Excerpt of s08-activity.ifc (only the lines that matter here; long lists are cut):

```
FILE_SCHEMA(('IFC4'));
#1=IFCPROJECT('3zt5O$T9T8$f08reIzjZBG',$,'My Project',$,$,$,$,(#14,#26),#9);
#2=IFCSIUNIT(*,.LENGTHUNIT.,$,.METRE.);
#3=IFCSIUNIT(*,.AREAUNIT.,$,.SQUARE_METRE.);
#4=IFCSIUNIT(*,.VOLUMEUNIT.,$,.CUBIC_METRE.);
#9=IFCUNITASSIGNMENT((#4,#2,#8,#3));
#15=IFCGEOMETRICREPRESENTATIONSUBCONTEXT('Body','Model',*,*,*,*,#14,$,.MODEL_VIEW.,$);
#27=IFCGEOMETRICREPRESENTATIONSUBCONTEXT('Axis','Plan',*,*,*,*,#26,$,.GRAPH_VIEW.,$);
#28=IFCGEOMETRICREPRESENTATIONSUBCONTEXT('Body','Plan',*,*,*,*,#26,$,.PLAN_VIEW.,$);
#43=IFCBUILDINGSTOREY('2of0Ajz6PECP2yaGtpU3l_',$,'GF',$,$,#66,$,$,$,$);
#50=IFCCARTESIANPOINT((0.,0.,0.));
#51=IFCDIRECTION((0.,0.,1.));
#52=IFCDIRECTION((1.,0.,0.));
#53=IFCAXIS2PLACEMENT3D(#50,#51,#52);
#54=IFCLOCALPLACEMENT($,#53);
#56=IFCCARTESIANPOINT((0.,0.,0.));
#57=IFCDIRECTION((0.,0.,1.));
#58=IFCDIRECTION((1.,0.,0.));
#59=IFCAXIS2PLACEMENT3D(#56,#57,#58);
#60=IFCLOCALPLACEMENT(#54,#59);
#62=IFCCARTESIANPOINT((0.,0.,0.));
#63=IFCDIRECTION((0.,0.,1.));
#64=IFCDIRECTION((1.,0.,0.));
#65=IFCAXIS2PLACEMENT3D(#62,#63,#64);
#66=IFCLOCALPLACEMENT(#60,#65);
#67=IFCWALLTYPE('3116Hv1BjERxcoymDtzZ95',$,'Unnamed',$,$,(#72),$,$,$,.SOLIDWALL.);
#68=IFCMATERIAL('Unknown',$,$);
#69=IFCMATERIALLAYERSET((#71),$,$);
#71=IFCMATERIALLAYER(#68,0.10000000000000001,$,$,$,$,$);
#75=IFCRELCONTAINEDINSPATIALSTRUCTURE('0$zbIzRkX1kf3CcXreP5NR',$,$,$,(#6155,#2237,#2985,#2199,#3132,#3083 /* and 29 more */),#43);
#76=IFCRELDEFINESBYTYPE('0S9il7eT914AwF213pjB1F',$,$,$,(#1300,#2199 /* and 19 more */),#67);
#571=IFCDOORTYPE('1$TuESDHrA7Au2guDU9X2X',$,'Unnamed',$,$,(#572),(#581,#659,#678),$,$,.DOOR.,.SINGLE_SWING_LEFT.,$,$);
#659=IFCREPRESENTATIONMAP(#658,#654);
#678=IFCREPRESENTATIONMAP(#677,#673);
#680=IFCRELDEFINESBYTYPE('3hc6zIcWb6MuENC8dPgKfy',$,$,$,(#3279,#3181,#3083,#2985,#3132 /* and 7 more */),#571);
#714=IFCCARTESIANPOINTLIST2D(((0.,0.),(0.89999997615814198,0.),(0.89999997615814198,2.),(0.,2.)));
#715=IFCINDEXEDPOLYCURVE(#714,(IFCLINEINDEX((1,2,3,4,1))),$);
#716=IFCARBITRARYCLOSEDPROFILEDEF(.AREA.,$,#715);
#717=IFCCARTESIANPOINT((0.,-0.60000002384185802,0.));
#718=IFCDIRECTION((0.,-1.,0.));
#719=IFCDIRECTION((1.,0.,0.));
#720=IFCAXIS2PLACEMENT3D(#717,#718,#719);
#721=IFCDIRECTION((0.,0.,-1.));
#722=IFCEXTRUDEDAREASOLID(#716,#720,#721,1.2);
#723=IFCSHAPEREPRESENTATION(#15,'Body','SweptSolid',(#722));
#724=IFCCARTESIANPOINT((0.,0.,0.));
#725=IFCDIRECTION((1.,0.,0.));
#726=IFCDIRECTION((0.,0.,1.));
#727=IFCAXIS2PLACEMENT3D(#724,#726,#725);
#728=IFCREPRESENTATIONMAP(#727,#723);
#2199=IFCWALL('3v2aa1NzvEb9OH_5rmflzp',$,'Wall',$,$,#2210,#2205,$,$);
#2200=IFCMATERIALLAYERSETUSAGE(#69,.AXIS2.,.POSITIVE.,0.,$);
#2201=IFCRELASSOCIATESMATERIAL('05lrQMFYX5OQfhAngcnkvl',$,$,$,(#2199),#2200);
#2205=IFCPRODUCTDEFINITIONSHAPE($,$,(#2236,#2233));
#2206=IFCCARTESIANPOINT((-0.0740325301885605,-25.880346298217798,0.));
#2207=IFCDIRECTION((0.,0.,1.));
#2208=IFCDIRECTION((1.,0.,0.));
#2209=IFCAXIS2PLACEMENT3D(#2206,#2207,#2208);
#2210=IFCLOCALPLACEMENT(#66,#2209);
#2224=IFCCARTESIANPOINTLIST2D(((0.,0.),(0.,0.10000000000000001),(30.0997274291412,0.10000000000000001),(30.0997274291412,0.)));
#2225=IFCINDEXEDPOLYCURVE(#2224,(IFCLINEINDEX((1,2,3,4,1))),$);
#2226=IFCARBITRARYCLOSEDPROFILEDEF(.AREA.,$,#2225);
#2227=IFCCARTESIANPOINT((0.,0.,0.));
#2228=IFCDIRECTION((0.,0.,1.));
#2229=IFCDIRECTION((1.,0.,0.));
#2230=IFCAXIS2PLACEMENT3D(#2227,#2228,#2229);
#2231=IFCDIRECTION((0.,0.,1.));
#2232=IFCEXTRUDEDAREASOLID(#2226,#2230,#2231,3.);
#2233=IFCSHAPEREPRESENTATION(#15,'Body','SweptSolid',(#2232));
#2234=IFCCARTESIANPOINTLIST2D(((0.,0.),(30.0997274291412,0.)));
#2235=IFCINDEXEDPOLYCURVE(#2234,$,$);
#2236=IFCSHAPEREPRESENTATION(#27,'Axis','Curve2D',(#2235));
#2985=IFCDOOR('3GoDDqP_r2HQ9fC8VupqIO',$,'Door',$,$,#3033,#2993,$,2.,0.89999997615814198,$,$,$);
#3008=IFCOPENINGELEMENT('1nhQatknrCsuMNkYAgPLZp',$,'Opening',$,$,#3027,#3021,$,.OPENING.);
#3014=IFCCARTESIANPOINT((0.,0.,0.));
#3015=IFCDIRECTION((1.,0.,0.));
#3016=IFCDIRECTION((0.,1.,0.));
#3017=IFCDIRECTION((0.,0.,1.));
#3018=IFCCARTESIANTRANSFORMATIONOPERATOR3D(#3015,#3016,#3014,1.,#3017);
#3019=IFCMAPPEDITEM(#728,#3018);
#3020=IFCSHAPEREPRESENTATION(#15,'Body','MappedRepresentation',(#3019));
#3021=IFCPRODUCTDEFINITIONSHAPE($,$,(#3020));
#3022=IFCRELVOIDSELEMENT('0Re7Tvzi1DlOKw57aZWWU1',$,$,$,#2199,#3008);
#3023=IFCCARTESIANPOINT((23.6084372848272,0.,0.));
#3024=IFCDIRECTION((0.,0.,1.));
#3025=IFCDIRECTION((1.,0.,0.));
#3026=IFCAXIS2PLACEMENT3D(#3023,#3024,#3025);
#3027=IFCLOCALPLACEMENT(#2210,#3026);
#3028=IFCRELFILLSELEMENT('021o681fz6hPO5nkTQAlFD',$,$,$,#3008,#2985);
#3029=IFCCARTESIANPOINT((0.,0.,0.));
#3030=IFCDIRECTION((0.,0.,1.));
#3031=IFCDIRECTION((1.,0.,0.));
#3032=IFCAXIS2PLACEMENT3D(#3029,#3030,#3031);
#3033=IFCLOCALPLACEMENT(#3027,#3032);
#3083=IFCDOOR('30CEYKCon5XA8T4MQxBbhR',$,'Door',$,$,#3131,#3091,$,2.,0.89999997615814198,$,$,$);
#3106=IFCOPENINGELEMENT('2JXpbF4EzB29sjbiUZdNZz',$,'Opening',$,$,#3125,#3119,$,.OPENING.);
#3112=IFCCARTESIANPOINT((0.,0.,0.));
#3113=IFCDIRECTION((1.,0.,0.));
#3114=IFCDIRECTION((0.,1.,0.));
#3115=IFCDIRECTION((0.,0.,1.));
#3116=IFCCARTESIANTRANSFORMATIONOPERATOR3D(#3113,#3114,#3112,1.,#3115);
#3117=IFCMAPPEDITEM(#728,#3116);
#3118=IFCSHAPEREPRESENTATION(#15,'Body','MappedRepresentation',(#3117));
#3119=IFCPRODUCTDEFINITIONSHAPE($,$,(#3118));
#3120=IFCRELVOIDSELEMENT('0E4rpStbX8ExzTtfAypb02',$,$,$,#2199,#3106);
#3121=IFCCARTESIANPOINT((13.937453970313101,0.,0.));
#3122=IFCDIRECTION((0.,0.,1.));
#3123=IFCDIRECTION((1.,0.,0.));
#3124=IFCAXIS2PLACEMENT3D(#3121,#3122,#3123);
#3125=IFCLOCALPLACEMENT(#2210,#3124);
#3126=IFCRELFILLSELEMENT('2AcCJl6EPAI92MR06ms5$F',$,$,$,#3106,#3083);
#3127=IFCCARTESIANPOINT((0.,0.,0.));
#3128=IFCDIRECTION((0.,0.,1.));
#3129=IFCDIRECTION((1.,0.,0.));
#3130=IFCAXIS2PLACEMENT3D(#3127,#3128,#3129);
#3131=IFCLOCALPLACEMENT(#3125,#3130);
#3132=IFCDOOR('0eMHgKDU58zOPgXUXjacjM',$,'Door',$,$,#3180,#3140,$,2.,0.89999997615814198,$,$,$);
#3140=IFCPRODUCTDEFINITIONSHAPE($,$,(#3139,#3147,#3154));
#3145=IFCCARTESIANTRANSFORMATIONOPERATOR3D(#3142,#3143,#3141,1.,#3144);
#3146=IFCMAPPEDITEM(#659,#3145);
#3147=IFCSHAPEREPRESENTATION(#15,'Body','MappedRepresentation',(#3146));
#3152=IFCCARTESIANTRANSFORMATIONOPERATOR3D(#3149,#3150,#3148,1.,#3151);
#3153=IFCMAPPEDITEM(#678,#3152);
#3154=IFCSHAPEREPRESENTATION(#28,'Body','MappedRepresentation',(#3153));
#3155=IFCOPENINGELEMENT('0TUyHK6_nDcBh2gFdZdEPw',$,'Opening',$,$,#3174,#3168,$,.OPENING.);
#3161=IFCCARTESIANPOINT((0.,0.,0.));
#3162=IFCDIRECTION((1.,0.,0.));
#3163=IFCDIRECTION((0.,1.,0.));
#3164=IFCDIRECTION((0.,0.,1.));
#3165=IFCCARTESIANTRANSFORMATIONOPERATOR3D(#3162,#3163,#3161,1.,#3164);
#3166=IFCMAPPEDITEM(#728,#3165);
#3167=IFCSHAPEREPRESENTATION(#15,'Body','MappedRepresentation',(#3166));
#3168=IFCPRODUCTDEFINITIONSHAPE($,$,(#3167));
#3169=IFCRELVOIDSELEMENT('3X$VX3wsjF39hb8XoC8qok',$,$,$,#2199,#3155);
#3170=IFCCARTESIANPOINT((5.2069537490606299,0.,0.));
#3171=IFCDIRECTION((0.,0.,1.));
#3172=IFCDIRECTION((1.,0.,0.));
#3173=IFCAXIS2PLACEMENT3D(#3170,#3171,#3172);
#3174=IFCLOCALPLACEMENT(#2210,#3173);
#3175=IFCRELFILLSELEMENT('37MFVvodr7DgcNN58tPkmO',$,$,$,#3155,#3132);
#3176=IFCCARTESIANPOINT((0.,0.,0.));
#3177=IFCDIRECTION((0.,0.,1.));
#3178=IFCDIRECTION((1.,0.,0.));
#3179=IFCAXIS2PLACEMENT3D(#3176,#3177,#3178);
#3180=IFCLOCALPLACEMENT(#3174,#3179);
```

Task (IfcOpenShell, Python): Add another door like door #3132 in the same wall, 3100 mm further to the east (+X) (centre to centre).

```python
import ifcopenshell
import ifcopenshell.api.feature
import ifcopenshell.api.geometry
import ifcopenshell.api.root
import ifcopenshell.geom
import ifcopenshell.util.element
import ifcopenshell.util.placement
import ifcopenshell.util.shape
import ifcopenshell.util.unit

model = ifcopenshell.open("s08-activity.ifc")
unit_scale = ifcopenshell.util.unit.calculate_unit_scale(model)
settings = ifcopenshell.geom.settings()


def volume(element):
    """Net volume in cubic metres, openings subtracted."""
    shape = ifcopenshell.geom.create_shape(settings, element)
    return ifcopenshell.util.shape.get_volume(shape.geometry)


door = model.by_guid("0eMHgKDU58zOPgXUXjacjM")
opening = door.FillsVoids[0].RelatingOpeningElement
wall = opening.VoidsElements[0].RelatingBuildingElement
before = volume(wall)
shift = ifcopenshell.util.placement.get_local_placement(wall.ObjectPlacement)[:3, 0] * 3.1 / unit_scale

# copy_class copies the void relationship, type, container and properties, but no geometry.
new_opening = ifcopenshell.api.root.copy_class(model, product=opening)
new_opening.Representation = ifcopenshell.util.element.copy_deep(
    model, opening.Representation, exclude=["IfcGeometricRepresentationContext", "IfcRepresentationMap"]
)
new_door = ifcopenshell.api.root.copy_class(model, product=door)
new_door.Representation = ifcopenshell.util.element.copy_deep(
    model, door.Representation, exclude=["IfcGeometricRepresentationContext", "IfcRepresentationMap"]
)
ifcopenshell.api.feature.add_filling(model, opening=new_opening, element=new_door)

for old, new in ((opening, new_opening), (door, new_door)):
    matrix = ifcopenshell.util.placement.get_local_placement(old.ObjectPlacement)
    matrix[:3, 3] += shift
    ifcopenshell.api.geometry.edit_object_placement(model, product=new, matrix=matrix, is_si=False)

after = volume(wall)

print(f"wall volume {before:.3f} -> {after:.3f} m3")

model.write("s08-activity-out.ifc")
```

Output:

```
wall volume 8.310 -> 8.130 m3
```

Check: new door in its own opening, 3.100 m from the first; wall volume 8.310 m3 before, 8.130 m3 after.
